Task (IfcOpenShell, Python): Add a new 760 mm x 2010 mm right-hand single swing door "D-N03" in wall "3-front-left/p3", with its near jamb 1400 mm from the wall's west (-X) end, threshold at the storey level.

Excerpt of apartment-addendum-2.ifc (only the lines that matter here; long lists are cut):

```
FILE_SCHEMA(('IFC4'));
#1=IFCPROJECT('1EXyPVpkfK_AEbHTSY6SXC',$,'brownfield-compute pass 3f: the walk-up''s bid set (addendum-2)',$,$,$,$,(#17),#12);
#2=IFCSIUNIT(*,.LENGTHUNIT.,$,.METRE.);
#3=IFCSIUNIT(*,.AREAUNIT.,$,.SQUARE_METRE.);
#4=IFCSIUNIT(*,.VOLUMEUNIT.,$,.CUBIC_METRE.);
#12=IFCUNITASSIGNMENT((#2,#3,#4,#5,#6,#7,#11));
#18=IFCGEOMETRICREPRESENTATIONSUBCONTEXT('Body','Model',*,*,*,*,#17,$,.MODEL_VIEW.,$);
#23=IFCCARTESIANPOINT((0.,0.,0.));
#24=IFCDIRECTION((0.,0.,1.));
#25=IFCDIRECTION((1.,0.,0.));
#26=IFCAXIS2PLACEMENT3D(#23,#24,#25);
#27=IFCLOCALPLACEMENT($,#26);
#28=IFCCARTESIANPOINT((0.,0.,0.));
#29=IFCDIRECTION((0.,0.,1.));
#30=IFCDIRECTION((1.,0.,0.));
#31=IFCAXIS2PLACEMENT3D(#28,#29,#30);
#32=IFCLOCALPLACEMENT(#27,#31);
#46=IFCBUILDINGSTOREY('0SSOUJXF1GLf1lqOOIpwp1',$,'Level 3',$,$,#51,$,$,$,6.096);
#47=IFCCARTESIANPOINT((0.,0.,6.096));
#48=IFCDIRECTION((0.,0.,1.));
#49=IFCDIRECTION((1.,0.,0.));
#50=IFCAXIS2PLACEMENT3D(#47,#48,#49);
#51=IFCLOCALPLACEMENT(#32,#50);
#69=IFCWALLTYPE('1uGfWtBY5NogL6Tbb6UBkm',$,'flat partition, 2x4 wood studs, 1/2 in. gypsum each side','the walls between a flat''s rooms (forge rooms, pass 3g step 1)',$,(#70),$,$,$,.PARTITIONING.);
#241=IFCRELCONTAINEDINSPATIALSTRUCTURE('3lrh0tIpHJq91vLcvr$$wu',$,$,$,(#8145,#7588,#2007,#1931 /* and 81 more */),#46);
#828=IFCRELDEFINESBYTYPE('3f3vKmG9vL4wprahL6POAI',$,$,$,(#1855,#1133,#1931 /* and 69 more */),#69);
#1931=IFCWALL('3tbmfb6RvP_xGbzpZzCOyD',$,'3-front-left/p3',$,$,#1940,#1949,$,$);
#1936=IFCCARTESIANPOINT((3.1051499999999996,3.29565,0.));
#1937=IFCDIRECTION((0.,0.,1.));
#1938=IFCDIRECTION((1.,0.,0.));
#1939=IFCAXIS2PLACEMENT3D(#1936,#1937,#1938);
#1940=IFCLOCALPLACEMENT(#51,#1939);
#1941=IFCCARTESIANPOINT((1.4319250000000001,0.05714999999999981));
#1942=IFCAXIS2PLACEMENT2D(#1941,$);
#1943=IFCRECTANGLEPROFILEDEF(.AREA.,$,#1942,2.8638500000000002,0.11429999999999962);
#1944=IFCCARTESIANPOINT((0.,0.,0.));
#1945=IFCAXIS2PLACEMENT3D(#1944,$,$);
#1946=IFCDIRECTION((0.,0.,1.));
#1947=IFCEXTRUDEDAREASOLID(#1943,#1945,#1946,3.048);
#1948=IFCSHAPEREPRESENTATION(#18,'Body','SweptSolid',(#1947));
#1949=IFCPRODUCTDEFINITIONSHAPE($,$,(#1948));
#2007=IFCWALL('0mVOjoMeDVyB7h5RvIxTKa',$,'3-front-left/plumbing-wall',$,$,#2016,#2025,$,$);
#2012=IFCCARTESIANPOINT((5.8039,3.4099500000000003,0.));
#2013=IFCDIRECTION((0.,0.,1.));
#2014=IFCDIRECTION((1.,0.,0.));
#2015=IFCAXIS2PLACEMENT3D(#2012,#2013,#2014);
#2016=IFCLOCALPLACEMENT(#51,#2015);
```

```python
import numpy as np
import ifcopenshell
import ifcopenshell.api.feature
import ifcopenshell.api.geometry
import ifcopenshell.api.root
import ifcopenshell.api.spatial
import ifcopenshell.geom
import ifcopenshell.util.element
import ifcopenshell.util.placement
import ifcopenshell.util.representation
import ifcopenshell.util.shape
import ifcopenshell.util.unit

model = ifcopenshell.open("apartment-addendum-2.ifc")
unit_scale = ifcopenshell.util.unit.calculate_unit_scale(model)
settings = ifcopenshell.geom.settings()


def volume(element):
    """Net volume in cubic metres, openings subtracted."""
    shape = ifcopenshell.geom.create_shape(settings, element)
    return ifcopenshell.util.shape.get_volume(shape.geometry)


wall = model.by_id(1931)
storey = ifcopenshell.util.element.get_container(wall, ifc_class="IfcBuildingStorey")
context = ifcopenshell.util.representation.get_context(model, "Model", "Body", "MODEL_VIEW")
before = volume(wall)

width, height, from_end, sill = 0.76, 2.01, 1.4, 0.0  # metres

# The wall runs along its own X axis, and the end named is its -X end.
wall_shape = ifcopenshell.geom.create_shape(settings, wall)
x, y, z = ifcopenshell.util.shape.get_vertices(wall_shape.geometry).T
start = x.min() + from_end
face, thickness = float(y.min()), float(y.max() - y.min())
wall_matrix = ifcopenshell.util.placement.get_local_placement(wall.ObjectPlacement)
level = ifcopenshell.util.placement.get_local_placement(storey.ObjectPlacement)[2, 3]


def in_wall(x, y):
    """Placement at x, y metres in the wall's axes, at sill height."""
    matrix = wall_matrix.copy()
    matrix[:, 3] = wall_matrix @ np.array([x / unit_scale, y / unit_scale, 0.0, 1.0])
    matrix[2, 3] = level + sill / unit_scale
    return matrix


# Opening: a box that overshoots both wall faces by 50 mm.
opening = ifcopenshell.api.root.create_entity(model, ifc_class="IfcOpeningElement", predefined_type="OPENING")
box = ifcopenshell.api.geometry.add_wall_representation(
    model, context=context, length=width, height=height, thickness=thickness + 0.1
)
ifcopenshell.api.geometry.assign_representation(model, product=opening, representation=box)
ifcopenshell.api.geometry.edit_object_placement(model, product=opening, matrix=in_wall(start, face - 0.05), is_si=False)
ifcopenshell.api.feature.add_feature(model, feature=opening, element=wall)

door = ifcopenshell.api.root.create_entity(model, ifc_class="IfcDoor", name="D-N03", predefined_type="DOOR")
door.OverallWidth, door.OverallHeight = width / unit_scale, height / unit_scale
door.OperationType = "SINGLE_SWING_RIGHT"
body = ifcopenshell.api.geometry.add_door_representation(
    model,
    context=context,
    overall_width=door.OverallWidth,
    overall_height=door.OverallHeight,
    operation_type="SINGLE_SWING_RIGHT",
    lining_properties={"LiningDepth": thickness / unit_scale, "ThresholdDepth": thickness / unit_scale},
)
ifcopenshell.api.geometry.assign_representation(model, product=door, representation=body)
ifcopenshell.api.spatial.assign_container(model, products=[door], relating_structure=storey)
ifcopenshell.api.feature.add_filling(model, opening=opening, element=door)

# The lining spans the wall, so the door starts at the wall face.
ifcopenshell.api.geometry.edit_object_placement(model, product=door, matrix=in_wall(start, face), is_si=False)

after = volume(wall)

print(f"wall volume {before:.3f} -> {after:.3f} m3")

model.write("apartment-addendum-2-out.ifc")
```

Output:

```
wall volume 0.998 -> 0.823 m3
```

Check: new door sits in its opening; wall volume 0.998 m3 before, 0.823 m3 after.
